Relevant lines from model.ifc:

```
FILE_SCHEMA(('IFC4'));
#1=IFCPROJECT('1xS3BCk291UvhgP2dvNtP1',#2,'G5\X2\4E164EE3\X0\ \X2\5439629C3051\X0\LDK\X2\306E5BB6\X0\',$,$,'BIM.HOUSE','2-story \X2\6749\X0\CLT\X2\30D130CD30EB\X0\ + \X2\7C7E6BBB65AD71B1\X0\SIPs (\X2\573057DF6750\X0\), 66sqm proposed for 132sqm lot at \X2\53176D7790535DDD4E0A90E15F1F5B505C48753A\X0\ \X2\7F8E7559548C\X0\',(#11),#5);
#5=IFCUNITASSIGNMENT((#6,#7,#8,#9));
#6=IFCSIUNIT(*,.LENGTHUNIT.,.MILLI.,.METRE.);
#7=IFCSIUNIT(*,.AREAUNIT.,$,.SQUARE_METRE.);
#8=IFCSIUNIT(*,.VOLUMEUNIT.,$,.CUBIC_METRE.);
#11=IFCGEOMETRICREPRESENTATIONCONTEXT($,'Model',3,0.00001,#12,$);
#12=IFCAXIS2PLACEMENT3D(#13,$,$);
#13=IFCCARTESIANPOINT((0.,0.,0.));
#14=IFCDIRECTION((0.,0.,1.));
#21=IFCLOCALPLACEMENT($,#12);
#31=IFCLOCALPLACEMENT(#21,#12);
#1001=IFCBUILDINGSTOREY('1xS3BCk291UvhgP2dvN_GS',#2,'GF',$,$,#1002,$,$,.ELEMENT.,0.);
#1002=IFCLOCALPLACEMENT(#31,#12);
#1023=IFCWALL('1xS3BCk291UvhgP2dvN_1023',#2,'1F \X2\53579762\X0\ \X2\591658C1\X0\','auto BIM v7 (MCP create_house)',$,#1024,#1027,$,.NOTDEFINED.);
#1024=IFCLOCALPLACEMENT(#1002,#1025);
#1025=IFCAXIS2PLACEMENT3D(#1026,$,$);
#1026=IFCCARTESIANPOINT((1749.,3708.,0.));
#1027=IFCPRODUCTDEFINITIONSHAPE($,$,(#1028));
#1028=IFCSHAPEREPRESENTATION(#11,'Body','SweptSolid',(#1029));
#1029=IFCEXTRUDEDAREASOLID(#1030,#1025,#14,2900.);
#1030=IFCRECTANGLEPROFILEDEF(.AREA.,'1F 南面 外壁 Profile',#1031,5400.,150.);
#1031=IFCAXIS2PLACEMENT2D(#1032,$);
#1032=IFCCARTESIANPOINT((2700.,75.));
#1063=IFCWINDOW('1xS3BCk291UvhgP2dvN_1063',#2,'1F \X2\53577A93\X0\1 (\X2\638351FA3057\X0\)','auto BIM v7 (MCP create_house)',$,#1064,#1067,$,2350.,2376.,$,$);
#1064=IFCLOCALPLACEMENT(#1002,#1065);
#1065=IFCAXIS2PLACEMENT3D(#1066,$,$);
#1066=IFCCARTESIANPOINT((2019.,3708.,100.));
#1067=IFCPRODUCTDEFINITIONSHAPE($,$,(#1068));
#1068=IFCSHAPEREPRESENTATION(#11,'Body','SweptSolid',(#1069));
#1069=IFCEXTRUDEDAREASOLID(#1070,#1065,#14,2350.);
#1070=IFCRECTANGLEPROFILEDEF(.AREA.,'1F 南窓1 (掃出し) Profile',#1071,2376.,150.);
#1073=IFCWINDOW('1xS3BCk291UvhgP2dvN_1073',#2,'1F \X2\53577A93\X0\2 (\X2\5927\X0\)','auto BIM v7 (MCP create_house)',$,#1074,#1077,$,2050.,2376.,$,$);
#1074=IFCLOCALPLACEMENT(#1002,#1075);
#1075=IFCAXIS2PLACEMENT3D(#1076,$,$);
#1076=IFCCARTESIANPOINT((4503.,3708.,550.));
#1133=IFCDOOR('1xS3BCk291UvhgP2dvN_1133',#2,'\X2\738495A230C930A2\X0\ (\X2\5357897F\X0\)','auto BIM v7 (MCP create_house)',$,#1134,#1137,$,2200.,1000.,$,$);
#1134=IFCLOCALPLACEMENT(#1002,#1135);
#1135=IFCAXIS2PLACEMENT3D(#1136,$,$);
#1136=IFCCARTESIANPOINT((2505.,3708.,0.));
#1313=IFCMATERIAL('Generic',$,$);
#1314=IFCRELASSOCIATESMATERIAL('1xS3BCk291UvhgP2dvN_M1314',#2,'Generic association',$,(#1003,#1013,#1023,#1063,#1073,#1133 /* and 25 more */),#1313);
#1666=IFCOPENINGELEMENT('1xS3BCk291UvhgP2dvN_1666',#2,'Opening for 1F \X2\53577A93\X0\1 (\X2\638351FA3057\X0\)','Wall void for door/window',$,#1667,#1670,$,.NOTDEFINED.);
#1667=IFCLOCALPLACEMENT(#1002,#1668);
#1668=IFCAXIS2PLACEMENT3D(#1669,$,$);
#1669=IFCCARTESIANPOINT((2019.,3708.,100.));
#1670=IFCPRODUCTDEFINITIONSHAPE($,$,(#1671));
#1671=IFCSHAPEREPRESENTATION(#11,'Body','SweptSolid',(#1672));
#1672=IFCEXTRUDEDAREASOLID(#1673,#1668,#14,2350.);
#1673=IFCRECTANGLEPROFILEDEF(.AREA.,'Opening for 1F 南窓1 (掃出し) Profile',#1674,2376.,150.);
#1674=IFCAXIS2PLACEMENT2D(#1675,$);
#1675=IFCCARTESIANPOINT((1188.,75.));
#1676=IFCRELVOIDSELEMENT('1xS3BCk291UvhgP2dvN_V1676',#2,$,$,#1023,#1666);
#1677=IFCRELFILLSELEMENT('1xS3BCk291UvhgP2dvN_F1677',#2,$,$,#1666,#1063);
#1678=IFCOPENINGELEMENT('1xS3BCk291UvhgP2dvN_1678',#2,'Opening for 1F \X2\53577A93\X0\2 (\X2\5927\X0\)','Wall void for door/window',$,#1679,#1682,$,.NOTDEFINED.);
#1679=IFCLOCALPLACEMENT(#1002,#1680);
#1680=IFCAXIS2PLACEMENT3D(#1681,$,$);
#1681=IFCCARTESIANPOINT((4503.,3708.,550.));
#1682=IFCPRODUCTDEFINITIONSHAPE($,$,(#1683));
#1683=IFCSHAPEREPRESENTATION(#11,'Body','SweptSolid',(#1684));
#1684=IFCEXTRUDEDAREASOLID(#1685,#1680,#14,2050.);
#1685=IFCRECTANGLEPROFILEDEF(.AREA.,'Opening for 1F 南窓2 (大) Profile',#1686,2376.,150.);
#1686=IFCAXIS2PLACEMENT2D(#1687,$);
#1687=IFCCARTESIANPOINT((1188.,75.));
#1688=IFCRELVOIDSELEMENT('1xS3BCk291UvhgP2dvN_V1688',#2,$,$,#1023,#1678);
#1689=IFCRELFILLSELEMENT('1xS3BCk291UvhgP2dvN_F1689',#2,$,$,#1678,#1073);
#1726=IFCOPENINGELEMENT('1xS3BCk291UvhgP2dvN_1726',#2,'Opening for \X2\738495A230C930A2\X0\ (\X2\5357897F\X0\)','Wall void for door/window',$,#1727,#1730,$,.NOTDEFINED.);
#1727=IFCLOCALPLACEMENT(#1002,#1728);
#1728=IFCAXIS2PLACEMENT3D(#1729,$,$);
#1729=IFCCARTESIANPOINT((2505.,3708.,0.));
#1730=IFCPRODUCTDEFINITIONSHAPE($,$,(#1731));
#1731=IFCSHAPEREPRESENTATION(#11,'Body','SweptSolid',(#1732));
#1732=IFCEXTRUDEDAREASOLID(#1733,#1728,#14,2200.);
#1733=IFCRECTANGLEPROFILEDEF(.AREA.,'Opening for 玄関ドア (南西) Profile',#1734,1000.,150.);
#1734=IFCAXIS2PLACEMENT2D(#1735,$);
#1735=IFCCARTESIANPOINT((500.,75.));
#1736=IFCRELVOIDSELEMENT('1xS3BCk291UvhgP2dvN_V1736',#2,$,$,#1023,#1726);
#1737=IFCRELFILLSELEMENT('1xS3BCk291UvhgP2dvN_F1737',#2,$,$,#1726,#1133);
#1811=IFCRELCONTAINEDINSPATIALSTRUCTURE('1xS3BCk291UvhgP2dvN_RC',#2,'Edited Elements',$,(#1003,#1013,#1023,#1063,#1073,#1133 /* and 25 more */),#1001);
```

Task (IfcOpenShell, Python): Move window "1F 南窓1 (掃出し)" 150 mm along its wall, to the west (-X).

```python
import ifcopenshell
import ifcopenshell.api.geometry
import ifcopenshell.util.placement
import ifcopenshell.util.unit

model = ifcopenshell.open("model.ifc")
unit_scale = ifcopenshell.util.unit.calculate_unit_scale(model)

window = model.by_id(1063)
opening = window.FillsVoids[0].RelatingOpeningElement
wall = opening.VoidsElements[0].RelatingBuildingElement

wall_matrix = ifcopenshell.util.placement.get_local_placement(wall.ObjectPlacement)
shift = wall_matrix[:3, 0] * -0.15 / unit_scale
before = ifcopenshell.util.placement.get_local_placement(window.ObjectPlacement)[:3, 3].copy()

# The window is not placed relative to its opening, so move both.
for product in (opening, window):
    matrix = ifcopenshell.util.placement.get_local_placement(product.ObjectPlacement)
    matrix[:3, 3] += shift
    ifcopenshell.api.geometry.edit_object_placement(model, product=product, matrix=matrix, is_si=False)

after = ifcopenshell.util.placement.get_local_placement(window.ObjectPlacement)[:3, 3]
print("window moved by", (after - before).round(3) + 0.0)

model.write("model-out.ifc")
```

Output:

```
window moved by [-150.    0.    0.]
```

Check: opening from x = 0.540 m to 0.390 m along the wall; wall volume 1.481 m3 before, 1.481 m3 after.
